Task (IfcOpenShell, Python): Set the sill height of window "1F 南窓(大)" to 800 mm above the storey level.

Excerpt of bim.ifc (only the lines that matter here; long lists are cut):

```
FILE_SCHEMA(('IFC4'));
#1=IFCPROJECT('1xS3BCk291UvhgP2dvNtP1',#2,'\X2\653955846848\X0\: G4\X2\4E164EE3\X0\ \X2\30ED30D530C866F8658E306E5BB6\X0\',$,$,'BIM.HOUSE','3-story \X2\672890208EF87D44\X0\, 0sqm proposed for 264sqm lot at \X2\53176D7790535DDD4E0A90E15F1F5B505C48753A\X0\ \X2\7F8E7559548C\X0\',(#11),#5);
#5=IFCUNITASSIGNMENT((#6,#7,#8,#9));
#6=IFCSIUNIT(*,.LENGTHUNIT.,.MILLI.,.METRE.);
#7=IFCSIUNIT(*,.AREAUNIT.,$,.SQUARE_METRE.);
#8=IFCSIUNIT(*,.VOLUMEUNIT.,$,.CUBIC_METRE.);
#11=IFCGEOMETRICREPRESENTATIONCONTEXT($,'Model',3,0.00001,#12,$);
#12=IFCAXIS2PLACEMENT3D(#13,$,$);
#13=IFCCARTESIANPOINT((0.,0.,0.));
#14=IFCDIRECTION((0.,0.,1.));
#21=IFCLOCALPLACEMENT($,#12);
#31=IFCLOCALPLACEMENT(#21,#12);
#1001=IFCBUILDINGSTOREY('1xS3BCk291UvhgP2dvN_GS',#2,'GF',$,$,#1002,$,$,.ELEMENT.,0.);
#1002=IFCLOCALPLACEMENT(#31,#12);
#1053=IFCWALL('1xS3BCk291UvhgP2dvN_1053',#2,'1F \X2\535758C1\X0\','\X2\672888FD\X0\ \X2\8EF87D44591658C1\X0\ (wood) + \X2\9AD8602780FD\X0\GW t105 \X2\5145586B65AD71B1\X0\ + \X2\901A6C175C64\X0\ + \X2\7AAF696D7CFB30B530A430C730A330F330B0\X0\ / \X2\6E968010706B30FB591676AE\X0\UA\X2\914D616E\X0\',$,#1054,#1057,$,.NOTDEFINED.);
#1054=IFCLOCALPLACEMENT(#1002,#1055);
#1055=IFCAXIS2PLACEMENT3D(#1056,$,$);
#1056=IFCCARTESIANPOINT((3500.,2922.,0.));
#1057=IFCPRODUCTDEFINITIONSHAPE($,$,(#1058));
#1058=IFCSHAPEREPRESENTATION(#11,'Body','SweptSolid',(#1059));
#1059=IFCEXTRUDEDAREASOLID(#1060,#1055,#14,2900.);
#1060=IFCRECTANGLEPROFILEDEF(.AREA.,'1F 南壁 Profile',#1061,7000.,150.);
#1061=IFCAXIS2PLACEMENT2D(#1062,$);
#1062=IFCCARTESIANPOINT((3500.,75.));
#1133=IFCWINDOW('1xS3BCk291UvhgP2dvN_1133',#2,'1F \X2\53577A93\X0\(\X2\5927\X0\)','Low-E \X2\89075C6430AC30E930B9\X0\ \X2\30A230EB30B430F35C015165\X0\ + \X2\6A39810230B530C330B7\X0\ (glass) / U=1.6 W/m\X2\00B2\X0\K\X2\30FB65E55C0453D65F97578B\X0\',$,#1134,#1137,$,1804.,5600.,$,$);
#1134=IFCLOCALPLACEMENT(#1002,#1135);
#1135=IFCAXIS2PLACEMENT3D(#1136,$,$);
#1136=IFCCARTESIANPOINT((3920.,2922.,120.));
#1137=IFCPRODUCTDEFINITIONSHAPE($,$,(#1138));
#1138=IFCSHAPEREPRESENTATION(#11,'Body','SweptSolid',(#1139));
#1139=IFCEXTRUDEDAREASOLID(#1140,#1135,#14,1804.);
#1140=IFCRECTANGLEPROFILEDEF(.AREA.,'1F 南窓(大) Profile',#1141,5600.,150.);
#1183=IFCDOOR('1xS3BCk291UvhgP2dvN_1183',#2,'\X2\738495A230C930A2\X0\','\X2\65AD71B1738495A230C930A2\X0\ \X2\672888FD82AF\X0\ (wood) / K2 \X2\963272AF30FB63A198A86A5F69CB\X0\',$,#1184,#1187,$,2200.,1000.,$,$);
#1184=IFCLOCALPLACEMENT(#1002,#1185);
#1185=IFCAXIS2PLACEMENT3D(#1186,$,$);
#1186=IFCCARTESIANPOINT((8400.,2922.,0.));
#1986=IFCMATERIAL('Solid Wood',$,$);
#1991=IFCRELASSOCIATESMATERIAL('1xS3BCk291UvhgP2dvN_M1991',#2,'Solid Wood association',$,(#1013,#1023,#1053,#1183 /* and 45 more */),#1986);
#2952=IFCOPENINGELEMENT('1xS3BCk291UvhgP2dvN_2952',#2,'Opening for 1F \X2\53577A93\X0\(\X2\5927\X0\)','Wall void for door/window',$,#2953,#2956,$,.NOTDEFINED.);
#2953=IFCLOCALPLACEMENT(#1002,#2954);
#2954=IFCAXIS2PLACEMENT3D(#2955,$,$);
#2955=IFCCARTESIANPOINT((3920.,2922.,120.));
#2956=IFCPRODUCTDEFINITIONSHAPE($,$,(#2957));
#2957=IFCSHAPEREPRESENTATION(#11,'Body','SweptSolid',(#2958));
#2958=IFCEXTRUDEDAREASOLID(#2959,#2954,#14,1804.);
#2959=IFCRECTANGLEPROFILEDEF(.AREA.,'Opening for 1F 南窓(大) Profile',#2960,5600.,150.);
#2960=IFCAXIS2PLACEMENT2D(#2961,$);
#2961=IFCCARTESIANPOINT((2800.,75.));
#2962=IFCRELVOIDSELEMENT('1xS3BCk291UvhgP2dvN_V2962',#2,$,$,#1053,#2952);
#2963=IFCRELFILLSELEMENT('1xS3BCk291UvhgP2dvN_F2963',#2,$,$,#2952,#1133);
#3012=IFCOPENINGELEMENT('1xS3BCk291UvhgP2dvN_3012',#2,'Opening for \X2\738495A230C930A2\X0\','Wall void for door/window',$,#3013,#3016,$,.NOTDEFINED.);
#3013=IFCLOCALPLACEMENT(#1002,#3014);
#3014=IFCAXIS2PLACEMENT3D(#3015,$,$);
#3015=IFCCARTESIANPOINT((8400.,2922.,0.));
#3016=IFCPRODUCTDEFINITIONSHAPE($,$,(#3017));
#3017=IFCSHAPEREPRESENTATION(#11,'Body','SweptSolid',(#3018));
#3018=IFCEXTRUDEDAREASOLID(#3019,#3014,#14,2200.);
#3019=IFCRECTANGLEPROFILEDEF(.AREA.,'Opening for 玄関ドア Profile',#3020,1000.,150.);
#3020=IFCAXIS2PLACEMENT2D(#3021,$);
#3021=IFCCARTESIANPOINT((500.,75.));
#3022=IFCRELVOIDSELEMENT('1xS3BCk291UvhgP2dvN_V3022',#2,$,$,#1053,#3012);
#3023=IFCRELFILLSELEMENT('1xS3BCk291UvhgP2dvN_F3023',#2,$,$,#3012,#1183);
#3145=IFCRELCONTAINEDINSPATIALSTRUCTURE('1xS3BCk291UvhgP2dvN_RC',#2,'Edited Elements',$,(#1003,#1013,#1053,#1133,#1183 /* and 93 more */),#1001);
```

```python
import numpy as np
import ifcopenshell
import ifcopenshell.api.geometry
import ifcopenshell.geom
import ifcopenshell.util.element
import ifcopenshell.util.placement
import ifcopenshell.util.shape
import ifcopenshell.util.unit

model = ifcopenshell.open("bim.ifc")
unit_scale = ifcopenshell.util.unit.calculate_unit_scale(model)

window = model.by_id(1133)
opening = window.FillsVoids[0].RelatingOpeningElement
storey = ifcopenshell.util.element.get_container(window, ifc_class="IfcBuildingStorey")
level = ifcopenshell.util.placement.get_local_placement(storey.ObjectPlacement)[2, 3]

# The opening's origin need not be at the sill, so measure its lowest point.
shape = ifcopenshell.geom.create_shape(ifcopenshell.geom.settings(), opening)
bottom = ifcopenshell.util.shape.get_shape_bottom_elevation(shape, shape.geometry) / unit_scale
dz = level + 0.8 / unit_scale - bottom

shift = np.array([0.0, 0.0, dz])
# The window is not placed relative to its opening, so move both.
for product in (opening, window):
    matrix = ifcopenshell.util.placement.get_local_placement(product.ObjectPlacement)
    matrix[:3, 3] += shift
    ifcopenshell.api.geometry.edit_object_placement(model, product=product, matrix=matrix, is_si=False)

print(f"moved by {dz * unit_scale:+.3f} m")

model.write("bim-out.ifc")
```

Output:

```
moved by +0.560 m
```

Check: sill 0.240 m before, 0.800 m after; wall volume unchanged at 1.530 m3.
